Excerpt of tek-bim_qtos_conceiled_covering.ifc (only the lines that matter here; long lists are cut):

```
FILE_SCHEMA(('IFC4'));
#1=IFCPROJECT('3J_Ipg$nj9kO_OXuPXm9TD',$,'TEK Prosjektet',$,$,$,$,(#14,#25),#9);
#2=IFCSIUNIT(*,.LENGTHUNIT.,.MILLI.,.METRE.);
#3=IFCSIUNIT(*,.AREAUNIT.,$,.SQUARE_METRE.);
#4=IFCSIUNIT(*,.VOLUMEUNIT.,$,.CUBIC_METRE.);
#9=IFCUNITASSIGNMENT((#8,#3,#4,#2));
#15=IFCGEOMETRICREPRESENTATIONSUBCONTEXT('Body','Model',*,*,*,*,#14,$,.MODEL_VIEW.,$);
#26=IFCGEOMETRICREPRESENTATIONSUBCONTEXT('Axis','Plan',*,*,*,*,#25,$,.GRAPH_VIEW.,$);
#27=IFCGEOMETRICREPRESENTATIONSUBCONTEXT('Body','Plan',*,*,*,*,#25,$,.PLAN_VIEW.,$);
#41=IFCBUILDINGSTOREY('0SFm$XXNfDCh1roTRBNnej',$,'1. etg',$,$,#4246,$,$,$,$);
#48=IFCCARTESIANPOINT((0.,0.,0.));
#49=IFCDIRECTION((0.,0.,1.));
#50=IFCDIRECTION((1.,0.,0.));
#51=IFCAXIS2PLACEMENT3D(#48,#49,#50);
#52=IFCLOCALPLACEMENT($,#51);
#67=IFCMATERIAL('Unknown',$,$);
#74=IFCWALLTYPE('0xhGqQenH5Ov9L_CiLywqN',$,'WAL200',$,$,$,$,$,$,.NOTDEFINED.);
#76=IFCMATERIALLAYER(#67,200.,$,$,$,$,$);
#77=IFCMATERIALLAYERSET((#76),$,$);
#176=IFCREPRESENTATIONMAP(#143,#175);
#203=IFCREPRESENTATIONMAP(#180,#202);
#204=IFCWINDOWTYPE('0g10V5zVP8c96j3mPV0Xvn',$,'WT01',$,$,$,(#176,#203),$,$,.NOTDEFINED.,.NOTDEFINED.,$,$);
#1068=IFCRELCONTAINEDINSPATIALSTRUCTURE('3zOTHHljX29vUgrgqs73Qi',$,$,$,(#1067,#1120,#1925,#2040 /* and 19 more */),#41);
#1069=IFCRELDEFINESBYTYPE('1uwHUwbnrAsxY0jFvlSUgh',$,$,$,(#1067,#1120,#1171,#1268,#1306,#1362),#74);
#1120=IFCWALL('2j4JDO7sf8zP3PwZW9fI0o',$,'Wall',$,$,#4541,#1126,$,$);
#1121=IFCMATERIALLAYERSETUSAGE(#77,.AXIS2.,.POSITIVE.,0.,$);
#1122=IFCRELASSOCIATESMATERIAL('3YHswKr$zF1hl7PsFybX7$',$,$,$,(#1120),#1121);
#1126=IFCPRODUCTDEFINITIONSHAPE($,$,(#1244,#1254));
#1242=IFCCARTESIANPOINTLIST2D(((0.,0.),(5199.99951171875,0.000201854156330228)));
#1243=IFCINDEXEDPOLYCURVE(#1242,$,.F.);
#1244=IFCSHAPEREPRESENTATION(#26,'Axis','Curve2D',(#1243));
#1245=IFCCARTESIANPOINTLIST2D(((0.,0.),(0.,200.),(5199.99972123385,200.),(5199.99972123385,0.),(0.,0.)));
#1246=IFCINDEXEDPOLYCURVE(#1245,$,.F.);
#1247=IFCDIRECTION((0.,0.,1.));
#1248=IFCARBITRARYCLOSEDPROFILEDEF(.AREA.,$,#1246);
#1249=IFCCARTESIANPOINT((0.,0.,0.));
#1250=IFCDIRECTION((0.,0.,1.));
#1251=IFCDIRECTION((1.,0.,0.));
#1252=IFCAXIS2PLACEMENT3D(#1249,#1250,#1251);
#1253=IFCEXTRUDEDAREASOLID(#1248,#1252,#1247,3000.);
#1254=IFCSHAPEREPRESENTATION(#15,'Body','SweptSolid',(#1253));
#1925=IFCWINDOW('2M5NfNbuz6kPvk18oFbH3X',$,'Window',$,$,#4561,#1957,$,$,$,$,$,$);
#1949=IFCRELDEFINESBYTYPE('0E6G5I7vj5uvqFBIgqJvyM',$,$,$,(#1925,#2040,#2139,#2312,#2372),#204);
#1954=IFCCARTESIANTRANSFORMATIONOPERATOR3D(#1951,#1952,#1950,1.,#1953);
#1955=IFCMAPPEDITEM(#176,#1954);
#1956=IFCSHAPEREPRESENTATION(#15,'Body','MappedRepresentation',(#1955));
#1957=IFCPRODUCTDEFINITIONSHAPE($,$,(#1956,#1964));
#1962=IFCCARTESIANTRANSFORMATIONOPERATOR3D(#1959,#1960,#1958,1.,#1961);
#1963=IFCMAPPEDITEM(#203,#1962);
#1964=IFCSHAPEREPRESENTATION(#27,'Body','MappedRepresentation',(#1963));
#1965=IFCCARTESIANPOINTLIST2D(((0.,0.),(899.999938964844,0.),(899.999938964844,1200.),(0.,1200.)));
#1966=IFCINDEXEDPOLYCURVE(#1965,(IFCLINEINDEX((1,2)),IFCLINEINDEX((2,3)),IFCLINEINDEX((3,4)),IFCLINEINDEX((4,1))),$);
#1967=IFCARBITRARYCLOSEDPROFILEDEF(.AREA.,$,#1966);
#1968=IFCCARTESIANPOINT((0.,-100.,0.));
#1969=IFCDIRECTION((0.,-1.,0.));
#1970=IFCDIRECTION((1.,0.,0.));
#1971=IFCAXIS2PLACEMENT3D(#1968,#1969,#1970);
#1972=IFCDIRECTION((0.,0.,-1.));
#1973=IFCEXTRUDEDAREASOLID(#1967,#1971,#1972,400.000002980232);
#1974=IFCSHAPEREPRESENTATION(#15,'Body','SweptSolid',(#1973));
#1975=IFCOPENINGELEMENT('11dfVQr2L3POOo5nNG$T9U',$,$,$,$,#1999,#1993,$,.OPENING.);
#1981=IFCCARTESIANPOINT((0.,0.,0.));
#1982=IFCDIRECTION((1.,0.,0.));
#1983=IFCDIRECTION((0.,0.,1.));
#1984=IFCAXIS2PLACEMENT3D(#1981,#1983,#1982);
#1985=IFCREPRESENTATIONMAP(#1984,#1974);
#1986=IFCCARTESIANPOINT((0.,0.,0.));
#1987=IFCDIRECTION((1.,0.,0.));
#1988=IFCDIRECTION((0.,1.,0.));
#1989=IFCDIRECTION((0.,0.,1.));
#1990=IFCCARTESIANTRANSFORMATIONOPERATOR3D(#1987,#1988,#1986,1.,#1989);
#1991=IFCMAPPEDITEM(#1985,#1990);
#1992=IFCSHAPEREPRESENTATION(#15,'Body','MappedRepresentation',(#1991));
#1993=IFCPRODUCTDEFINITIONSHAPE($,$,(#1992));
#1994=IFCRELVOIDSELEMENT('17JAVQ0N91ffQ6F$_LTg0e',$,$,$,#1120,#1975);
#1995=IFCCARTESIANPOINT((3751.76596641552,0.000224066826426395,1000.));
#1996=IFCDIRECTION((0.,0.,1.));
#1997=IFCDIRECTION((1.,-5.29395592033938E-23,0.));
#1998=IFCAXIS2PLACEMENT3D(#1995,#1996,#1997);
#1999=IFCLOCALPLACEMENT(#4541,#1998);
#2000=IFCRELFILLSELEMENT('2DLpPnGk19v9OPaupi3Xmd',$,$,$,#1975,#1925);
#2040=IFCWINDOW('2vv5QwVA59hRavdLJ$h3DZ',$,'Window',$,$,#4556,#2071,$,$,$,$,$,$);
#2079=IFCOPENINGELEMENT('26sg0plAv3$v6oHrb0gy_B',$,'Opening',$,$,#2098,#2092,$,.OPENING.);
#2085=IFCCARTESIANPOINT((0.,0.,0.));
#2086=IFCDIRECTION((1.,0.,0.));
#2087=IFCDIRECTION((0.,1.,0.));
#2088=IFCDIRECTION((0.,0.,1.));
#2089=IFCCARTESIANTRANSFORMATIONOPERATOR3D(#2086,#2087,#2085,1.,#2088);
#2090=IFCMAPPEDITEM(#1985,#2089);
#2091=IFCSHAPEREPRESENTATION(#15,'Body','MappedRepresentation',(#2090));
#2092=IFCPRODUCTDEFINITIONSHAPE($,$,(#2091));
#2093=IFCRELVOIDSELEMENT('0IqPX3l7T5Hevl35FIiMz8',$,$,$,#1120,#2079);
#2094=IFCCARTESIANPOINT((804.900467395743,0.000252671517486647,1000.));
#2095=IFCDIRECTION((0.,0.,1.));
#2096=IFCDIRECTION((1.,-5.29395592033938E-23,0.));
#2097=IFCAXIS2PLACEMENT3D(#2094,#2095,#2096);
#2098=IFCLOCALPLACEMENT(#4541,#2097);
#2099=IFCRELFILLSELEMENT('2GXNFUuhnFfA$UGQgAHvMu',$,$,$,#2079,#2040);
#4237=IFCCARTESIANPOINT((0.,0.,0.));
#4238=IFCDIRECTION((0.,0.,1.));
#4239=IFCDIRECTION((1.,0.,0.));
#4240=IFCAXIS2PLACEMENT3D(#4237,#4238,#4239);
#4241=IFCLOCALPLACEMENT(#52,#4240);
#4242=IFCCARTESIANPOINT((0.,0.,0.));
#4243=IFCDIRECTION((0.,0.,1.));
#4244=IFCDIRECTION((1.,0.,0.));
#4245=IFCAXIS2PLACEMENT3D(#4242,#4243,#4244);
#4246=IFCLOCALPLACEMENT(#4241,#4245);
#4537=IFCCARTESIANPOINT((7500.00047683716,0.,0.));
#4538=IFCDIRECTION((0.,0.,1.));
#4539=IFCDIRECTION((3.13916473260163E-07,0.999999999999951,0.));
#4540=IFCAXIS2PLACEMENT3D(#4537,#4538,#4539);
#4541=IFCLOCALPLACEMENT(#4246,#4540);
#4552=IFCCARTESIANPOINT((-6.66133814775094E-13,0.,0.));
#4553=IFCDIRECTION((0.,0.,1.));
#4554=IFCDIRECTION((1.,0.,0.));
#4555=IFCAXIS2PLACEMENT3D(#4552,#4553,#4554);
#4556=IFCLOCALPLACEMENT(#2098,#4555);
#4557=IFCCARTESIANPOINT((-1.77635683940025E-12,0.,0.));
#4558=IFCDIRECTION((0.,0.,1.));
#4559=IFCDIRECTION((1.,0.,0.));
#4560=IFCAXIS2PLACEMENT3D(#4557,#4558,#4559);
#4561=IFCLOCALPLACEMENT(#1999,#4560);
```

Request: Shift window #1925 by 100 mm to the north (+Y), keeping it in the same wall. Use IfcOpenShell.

```python
import ifcopenshell
import ifcopenshell.api.geometry
import ifcopenshell.util.placement
import ifcopenshell.util.unit

model = ifcopenshell.open("tek-bim_qtos_conceiled_covering.ifc")
unit_scale = ifcopenshell.util.unit.calculate_unit_scale(model)

window = model.by_guid("2M5NfNbuz6kPvk18oFbH3X")
opening = window.FillsVoids[0].RelatingOpeningElement
wall = opening.VoidsElements[0].RelatingBuildingElement

wall_matrix = ifcopenshell.util.placement.get_local_placement(wall.ObjectPlacement)
shift = wall_matrix[:3, 0] * 0.1 / unit_scale
before = ifcopenshell.util.placement.get_local_placement(window.ObjectPlacement)[:3, 3].copy()

# The window is placed relative to its opening, so it follows when the opening moves.
matrix = ifcopenshell.util.placement.get_local_placement(opening.ObjectPlacement)
matrix[:3, 3] += shift
ifcopenshell.api.geometry.edit_object_placement(
    model, product=opening, matrix=matrix, is_si=False, should_transform_children=True
)

after = ifcopenshell.util.placement.get_local_placement(window.ObjectPlacement)[:3, 3]
print("window moved by", (after - before).round(3) + 0.0)

model.write("tek-bim_qtos_conceiled_covering-out.ifc")
```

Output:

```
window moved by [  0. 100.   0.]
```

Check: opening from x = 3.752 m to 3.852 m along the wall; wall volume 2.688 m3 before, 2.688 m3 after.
